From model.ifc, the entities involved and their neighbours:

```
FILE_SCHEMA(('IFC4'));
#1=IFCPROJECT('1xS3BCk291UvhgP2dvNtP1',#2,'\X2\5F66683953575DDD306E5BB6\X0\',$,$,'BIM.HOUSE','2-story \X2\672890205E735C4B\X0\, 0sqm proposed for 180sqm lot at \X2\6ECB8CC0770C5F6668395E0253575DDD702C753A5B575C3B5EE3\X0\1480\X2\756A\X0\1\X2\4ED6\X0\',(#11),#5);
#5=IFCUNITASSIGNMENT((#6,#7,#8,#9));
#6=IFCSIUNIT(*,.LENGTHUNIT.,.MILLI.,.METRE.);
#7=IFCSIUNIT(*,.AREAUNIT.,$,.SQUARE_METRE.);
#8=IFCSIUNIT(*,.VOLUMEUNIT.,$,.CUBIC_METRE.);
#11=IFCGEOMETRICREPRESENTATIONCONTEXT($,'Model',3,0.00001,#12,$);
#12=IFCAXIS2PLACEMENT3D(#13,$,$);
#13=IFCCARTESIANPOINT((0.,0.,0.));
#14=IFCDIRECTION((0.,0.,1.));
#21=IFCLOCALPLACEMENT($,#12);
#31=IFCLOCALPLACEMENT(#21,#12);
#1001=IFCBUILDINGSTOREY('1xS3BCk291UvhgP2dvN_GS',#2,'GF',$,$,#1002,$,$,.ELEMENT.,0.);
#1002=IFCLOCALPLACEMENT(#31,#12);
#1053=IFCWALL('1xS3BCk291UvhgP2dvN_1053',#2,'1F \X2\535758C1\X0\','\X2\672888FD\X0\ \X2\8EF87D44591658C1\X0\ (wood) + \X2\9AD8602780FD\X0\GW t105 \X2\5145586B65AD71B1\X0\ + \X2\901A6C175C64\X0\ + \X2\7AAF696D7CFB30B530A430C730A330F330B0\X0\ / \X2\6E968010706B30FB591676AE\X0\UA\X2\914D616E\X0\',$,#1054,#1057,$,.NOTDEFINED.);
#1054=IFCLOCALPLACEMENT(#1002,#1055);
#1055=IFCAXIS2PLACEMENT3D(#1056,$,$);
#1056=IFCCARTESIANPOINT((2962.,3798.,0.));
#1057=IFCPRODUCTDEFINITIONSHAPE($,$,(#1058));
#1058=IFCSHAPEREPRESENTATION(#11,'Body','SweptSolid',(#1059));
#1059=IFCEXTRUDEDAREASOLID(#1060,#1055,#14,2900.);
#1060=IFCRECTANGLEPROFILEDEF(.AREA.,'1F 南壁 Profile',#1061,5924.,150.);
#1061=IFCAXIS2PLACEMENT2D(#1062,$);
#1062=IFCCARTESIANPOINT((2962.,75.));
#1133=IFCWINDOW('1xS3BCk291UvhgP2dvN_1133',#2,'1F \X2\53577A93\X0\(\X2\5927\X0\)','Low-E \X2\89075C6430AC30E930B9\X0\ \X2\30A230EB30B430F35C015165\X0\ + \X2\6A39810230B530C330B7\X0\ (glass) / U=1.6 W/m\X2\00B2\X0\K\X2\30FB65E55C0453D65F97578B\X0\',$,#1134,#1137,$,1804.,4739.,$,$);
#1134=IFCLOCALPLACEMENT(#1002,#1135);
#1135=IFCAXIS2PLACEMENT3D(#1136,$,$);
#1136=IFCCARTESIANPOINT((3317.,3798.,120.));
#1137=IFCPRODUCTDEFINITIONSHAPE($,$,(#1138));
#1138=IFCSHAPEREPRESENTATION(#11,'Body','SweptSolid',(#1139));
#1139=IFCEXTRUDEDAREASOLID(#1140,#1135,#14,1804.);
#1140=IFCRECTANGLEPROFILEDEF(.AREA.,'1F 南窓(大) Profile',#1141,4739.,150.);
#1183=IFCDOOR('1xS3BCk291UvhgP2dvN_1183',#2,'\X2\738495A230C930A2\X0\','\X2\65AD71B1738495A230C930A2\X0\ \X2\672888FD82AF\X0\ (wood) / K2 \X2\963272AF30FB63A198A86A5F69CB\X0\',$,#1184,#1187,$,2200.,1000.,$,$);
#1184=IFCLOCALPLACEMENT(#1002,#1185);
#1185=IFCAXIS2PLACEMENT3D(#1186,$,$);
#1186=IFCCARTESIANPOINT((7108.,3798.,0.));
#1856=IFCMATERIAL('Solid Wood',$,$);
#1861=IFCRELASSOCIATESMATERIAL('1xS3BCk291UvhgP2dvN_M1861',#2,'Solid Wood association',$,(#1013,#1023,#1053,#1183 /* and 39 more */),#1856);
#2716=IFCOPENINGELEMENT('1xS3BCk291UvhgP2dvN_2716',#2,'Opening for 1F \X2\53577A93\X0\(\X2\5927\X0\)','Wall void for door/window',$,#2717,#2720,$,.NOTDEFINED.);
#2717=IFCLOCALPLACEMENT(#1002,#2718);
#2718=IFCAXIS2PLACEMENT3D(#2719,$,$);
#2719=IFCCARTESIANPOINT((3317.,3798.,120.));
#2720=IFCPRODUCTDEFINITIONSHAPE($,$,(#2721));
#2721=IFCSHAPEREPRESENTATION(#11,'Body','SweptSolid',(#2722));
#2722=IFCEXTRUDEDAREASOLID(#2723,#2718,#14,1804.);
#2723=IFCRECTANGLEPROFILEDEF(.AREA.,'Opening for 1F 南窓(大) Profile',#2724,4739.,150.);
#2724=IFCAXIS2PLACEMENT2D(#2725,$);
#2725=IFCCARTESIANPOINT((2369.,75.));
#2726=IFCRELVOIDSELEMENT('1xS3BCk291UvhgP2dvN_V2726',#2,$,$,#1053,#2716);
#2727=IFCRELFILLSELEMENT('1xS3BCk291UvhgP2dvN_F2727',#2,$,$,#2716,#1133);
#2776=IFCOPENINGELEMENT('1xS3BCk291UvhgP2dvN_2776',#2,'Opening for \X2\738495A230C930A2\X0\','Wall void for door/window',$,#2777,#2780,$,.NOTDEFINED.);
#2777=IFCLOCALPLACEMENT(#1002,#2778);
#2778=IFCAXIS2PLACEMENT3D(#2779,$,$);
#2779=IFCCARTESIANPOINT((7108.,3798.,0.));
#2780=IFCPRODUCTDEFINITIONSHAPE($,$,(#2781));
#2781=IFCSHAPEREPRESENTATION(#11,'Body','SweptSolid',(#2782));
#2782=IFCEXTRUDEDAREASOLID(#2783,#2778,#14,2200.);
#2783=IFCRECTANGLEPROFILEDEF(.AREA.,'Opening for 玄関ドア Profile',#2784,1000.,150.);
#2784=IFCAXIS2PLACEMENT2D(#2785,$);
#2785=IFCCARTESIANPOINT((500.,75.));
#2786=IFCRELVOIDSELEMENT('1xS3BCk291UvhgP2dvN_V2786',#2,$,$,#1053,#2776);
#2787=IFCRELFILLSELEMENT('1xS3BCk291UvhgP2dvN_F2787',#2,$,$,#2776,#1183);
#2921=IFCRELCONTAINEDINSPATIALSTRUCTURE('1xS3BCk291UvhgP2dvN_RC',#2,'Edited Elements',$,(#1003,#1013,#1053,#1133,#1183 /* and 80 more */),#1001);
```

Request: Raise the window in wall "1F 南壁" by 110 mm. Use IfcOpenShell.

```python
import numpy as np
import ifcopenshell
import ifcopenshell.api.geometry
import ifcopenshell.util.placement
import ifcopenshell.util.unit

model = ifcopenshell.open("model.ifc")
unit_scale = ifcopenshell.util.unit.calculate_unit_scale(model)

window = model.by_guid("1xS3BCk291UvhgP2dvN_1133")
opening = window.FillsVoids[0].RelatingOpeningElement
dz = 0.11 / unit_scale

shift = np.array([0.0, 0.0, dz])
# The window is not placed relative to its opening, so move both.
for product in (opening, window):
    matrix = ifcopenshell.util.placement.get_local_placement(product.ObjectPlacement)
    matrix[:3, 3] += shift
    ifcopenshell.api.geometry.edit_object_placement(model, product=product, matrix=matrix, is_si=False)

print(f"moved by {dz * unit_scale:+.3f} m")

model.write("model_edited.ifc")
```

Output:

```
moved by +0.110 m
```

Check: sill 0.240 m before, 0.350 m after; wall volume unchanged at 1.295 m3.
